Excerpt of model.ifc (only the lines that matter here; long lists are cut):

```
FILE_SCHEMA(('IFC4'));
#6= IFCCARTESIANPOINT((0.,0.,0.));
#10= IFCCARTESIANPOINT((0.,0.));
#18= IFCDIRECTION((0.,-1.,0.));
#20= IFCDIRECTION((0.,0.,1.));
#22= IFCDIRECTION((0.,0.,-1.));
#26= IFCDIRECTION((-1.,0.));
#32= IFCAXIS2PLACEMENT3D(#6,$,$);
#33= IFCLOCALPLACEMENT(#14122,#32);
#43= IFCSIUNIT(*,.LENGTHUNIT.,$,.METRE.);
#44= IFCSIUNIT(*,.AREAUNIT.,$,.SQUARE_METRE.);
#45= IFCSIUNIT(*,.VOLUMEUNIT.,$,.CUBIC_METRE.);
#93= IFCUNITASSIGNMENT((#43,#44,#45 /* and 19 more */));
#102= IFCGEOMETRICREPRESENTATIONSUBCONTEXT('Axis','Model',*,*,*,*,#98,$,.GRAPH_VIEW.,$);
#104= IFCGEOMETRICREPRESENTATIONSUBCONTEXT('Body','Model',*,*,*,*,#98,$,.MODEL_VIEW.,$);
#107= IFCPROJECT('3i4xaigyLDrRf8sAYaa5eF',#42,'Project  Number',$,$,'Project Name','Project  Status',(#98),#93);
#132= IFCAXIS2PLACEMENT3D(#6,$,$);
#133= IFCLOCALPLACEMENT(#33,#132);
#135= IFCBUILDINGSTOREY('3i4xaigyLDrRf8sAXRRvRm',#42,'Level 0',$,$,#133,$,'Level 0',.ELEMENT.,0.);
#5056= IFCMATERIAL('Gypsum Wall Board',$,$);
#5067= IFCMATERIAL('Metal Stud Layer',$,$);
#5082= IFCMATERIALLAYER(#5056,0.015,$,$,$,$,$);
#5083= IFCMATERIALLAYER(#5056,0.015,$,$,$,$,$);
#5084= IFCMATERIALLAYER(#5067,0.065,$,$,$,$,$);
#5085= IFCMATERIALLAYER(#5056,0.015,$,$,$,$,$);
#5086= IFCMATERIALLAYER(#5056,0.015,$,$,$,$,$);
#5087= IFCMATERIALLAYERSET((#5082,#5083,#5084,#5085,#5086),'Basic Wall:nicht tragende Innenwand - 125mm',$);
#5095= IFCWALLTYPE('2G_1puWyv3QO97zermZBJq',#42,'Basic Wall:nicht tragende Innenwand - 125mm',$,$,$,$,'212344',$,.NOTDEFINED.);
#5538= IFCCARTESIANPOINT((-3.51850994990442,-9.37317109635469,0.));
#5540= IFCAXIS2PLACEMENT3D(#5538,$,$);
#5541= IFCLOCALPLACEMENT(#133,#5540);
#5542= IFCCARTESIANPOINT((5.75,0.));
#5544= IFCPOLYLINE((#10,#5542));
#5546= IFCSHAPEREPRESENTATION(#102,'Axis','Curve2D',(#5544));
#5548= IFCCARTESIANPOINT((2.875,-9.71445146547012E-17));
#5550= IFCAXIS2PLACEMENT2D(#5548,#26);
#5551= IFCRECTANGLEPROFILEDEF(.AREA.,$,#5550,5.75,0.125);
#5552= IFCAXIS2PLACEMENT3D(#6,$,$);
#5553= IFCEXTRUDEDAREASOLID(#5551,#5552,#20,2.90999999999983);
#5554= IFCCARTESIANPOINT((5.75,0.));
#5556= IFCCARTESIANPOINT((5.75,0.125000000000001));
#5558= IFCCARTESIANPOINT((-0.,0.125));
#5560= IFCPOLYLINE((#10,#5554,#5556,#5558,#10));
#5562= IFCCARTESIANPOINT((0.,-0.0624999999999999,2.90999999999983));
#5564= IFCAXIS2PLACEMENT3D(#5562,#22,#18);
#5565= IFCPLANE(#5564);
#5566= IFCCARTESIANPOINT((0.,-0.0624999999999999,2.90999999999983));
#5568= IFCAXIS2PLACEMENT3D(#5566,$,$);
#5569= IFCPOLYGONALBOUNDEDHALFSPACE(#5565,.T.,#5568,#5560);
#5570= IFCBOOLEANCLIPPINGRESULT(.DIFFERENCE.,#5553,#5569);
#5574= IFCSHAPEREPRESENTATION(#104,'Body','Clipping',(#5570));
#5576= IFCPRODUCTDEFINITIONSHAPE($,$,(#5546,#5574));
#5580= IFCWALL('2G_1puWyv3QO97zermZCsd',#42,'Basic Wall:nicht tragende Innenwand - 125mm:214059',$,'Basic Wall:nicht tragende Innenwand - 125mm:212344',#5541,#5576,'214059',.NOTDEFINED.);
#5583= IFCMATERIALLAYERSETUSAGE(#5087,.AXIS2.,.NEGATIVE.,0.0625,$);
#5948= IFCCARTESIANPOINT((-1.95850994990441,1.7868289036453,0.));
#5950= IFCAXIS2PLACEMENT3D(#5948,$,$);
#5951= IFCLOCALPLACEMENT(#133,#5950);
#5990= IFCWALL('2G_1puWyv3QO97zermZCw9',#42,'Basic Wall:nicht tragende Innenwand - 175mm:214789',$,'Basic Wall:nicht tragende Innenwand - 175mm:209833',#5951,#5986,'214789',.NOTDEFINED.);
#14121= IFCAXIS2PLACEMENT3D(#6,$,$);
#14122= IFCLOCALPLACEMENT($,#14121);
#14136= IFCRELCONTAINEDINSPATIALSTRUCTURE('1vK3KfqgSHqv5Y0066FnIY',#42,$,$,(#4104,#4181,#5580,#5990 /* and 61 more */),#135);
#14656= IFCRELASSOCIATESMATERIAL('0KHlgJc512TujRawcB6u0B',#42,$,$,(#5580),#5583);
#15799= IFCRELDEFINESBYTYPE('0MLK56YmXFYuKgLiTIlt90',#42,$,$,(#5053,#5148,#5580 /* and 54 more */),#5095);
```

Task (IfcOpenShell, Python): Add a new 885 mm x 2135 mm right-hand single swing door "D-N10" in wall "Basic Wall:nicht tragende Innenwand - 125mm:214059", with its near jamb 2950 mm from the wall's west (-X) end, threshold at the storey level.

```python
import numpy as np
import ifcopenshell
import ifcopenshell.api.feature
import ifcopenshell.api.geometry
import ifcopenshell.api.root
import ifcopenshell.api.spatial
import ifcopenshell.geom
import ifcopenshell.util.element
import ifcopenshell.util.placement
import ifcopenshell.util.representation
import ifcopenshell.util.shape
import ifcopenshell.util.unit

model = ifcopenshell.open("model.ifc")
unit_scale = ifcopenshell.util.unit.calculate_unit_scale(model)
settings = ifcopenshell.geom.settings()


def volume(element):
    """Net volume in cubic metres, openings subtracted."""
    shape = ifcopenshell.geom.create_shape(settings, element)
    return ifcopenshell.util.shape.get_volume(shape.geometry)


wall = model.by_id(5580)
storey = ifcopenshell.util.element.get_container(wall, ifc_class="IfcBuildingStorey")
context = ifcopenshell.util.representation.get_context(model, "Model", "Body", "MODEL_VIEW")
before = volume(wall)

width, height, from_end, sill = 0.885, 2.135, 2.95, 0.0  # metres

# The wall runs along its own X axis, and the end named is its -X end.
wall_shape = ifcopenshell.geom.create_shape(settings, wall)
x, y, z = ifcopenshell.util.shape.get_vertices(wall_shape.geometry).T
start = x.min() + from_end
face, thickness = float(y.min()), float(y.max() - y.min())
wall_matrix = ifcopenshell.util.placement.get_local_placement(wall.ObjectPlacement)
level = ifcopenshell.util.placement.get_local_placement(storey.ObjectPlacement)[2, 3]


def in_wall(x, y):
    """Placement at x, y metres in the wall's axes, at sill height."""
    matrix = wall_matrix.copy()
    matrix[:, 3] = wall_matrix @ np.array([x / unit_scale, y / unit_scale, 0.0, 1.0])
    matrix[2, 3] = level + sill / unit_scale
    return matrix


# Opening: a box that overshoots both wall faces by 50 mm.
opening = ifcopenshell.api.root.create_entity(model, ifc_class="IfcOpeningElement", predefined_type="OPENING")
box = ifcopenshell.api.geometry.add_wall_representation(
    model, context=context, length=width, height=height, thickness=thickness + 0.1
)
ifcopenshell.api.geometry.assign_representation(model, product=opening, representation=box)
ifcopenshell.api.geometry.edit_object_placement(model, product=opening, matrix=in_wall(start, face - 0.05), is_si=False)
ifcopenshell.api.feature.add_feature(model, feature=opening, element=wall)

door = ifcopenshell.api.root.create_entity(model, ifc_class="IfcDoor", name="D-N10", predefined_type="DOOR")
door.OverallWidth, door.OverallHeight = width / unit_scale, height / unit_scale
door.OperationType = "SINGLE_SWING_RIGHT"
body = ifcopenshell.api.geometry.add_door_representation(
    model,
    context=context,
    overall_width=door.OverallWidth,
    overall_height=door.OverallHeight,
    operation_type="SINGLE_SWING_RIGHT",
    lining_properties={"LiningDepth": thickness / unit_scale, "ThresholdDepth": thickness / unit_scale},
)
ifcopenshell.api.geometry.assign_representation(model, product=door, representation=body)
ifcopenshell.api.spatial.assign_container(model, products=[door], relating_structure=storey)
ifcopenshell.api.feature.add_filling(model, opening=opening, element=door)

# The lining spans the wall, so the door starts at the wall face.
ifcopenshell.api.geometry.edit_object_placement(model, product=door, matrix=in_wall(start, face), is_si=False)

after = volume(wall)

print(f"wall volume {before:.3f} -> {after:.3f} m3")

model.write("model_v2.ifc")
```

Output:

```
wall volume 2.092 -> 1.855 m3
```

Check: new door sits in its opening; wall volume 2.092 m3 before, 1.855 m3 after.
